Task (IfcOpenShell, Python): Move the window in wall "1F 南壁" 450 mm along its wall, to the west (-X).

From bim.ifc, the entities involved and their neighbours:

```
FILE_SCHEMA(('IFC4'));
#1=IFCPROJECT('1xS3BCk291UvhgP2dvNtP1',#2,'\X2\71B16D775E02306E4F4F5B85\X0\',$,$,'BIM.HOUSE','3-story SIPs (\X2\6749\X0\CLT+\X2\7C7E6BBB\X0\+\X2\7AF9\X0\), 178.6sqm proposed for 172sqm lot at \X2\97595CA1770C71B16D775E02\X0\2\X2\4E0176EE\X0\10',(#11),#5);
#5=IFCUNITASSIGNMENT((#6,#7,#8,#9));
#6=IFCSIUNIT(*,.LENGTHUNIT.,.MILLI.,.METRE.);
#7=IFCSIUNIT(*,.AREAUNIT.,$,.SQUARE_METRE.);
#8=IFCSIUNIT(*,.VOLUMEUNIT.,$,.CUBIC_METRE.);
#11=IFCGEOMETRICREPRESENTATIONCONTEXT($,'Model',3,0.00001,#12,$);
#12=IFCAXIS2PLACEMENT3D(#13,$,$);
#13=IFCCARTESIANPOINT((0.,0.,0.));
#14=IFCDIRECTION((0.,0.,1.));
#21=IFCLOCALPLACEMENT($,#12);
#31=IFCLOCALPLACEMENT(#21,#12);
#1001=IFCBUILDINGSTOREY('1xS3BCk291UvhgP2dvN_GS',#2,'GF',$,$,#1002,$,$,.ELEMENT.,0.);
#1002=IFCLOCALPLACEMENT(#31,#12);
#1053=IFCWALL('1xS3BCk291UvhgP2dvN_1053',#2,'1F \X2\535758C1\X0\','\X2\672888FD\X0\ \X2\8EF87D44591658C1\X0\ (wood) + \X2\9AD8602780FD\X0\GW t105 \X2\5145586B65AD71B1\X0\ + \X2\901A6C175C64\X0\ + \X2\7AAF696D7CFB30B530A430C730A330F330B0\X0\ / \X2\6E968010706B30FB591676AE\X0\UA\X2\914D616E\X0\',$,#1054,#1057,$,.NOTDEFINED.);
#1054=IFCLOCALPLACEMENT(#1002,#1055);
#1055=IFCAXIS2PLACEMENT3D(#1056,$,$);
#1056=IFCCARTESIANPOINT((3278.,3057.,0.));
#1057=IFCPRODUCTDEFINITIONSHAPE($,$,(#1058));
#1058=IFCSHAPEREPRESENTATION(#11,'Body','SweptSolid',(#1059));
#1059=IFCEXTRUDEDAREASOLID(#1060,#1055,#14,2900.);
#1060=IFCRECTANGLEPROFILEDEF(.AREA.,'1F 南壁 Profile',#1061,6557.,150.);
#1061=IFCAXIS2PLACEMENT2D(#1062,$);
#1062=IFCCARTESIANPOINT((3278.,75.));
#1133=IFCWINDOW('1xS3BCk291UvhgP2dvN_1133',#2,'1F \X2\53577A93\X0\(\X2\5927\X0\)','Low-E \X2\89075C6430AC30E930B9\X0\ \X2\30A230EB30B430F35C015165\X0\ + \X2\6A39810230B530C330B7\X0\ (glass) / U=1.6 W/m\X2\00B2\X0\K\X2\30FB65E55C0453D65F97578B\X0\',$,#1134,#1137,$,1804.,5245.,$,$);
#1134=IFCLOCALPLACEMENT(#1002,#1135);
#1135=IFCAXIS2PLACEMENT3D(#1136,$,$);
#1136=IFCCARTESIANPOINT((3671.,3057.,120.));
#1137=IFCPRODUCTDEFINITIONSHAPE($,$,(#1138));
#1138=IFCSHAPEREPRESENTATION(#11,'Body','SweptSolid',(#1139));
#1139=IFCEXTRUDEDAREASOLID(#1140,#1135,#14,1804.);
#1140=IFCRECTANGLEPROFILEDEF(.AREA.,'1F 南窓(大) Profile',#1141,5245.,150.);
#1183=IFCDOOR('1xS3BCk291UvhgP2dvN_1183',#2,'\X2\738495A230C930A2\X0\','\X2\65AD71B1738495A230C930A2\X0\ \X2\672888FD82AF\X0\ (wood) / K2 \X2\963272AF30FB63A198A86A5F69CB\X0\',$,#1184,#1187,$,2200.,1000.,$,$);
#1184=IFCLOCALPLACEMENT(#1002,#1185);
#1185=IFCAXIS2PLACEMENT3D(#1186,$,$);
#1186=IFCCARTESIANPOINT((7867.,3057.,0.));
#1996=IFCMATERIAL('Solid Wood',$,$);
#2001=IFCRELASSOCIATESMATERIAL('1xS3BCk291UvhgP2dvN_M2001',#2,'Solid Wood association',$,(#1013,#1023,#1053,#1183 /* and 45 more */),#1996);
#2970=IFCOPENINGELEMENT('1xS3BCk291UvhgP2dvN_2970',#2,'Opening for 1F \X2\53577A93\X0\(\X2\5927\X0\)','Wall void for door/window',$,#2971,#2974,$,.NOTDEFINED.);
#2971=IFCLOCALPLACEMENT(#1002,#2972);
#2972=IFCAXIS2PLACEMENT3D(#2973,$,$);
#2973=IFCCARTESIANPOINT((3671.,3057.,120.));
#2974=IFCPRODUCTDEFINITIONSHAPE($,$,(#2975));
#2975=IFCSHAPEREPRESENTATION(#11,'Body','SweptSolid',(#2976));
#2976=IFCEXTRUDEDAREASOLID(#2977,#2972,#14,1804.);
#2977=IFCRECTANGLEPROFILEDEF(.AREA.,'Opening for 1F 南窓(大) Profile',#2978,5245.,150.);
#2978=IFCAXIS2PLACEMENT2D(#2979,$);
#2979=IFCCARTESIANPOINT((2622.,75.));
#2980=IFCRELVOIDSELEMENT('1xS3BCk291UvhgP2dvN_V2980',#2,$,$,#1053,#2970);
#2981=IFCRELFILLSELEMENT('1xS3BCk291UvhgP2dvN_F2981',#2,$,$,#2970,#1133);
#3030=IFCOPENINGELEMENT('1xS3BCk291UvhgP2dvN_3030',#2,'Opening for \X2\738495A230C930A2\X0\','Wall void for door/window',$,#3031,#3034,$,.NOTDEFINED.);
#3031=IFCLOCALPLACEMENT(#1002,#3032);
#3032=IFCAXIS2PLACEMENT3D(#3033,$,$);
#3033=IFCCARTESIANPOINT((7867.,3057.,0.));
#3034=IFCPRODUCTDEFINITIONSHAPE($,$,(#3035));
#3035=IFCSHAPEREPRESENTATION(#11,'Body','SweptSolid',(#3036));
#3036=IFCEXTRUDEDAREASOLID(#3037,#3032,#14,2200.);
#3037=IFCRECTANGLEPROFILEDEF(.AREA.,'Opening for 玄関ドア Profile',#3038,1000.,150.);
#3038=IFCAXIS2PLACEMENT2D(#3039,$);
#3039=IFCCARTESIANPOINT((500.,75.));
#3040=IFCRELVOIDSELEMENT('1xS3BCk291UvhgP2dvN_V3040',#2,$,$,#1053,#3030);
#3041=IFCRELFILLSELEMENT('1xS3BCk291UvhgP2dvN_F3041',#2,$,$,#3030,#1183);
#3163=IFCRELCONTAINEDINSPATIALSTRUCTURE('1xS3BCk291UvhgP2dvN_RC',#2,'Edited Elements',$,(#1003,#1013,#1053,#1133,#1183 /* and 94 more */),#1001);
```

```python
import ifcopenshell
import ifcopenshell.api.geometry
import ifcopenshell.util.placement
import ifcopenshell.util.unit

model = ifcopenshell.open("bim.ifc")
unit_scale = ifcopenshell.util.unit.calculate_unit_scale(model)

window = model.by_guid("1xS3BCk291UvhgP2dvN_1133")
opening = window.FillsVoids[0].RelatingOpeningElement
wall = opening.VoidsElements[0].RelatingBuildingElement

wall_matrix = ifcopenshell.util.placement.get_local_placement(wall.ObjectPlacement)
shift = wall_matrix[:3, 0] * -0.45 / unit_scale
before = ifcopenshell.util.placement.get_local_placement(window.ObjectPlacement)[:3, 3].copy()

# The window is not placed relative to its opening, so move both.
for product in (opening, window):
    matrix = ifcopenshell.util.placement.get_local_placement(product.ObjectPlacement)
    matrix[:3, 3] += shift
    ifcopenshell.api.geometry.edit_object_placement(model, product=product, matrix=matrix, is_si=False)

after = ifcopenshell.util.placement.get_local_placement(window.ObjectPlacement)[:3, 3]
print("window moved by", (after - before).round(3) + 0.0)

model.write("bim_updated.ifc")
```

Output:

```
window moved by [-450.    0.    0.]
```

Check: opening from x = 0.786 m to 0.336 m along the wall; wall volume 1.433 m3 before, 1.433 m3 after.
